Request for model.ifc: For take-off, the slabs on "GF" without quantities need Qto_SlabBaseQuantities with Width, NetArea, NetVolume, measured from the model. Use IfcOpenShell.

First a look at what the model holds.

```python
import ifcopenshell
import ifcopenshell.util.element
import ifcopenshell.util.unit

model = ifcopenshell.open("model.ifc")
print(model.schema)
for unit_type in ("LENGTHUNIT", "AREAUNIT", "VOLUMEUNIT"):
    print(unit_type, ifcopenshell.util.unit.calculate_unit_scale(model, unit_type))
storey = next(s for s in model.by_type("IfcBuildingStorey") if s.Name == "GF")
slabs = [e for e in ifcopenshell.util.element.get_decomposition(storey) if e.is_a("IfcSlab")]
for e in sorted(slabs, key=lambda e: e.id()):
    print(e.id(), e.is_a(), e.Name, list(ifcopenshell.util.element.get_psets(e, qtos_only=True)), sep=" | ")
```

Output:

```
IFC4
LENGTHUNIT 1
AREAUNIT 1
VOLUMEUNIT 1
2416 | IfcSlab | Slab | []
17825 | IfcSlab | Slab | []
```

```python
import ifcopenshell
import ifcopenshell.api.pset
import ifcopenshell.geom
import ifcopenshell.util.element
import ifcopenshell.util.shape
import ifcopenshell.util.unit

model = ifcopenshell.open("model.ifc")
unit_scale = ifcopenshell.util.unit.calculate_unit_scale(model)
area_scale = ifcopenshell.util.unit.calculate_unit_scale(model, "AREAUNIT")
volume_scale = ifcopenshell.util.unit.calculate_unit_scale(model, "VOLUMEUNIT")
settings = ifcopenshell.geom.settings()

storey = next(s for s in model.by_type("IfcBuildingStorey") if s.Name == "GF")
slabs = [e for e in ifcopenshell.util.element.get_decomposition(storey) if e.is_a("IfcSlab")]

for e in sorted(slabs, key=lambda e: e.id()):
    if ifcopenshell.util.element.get_psets(e, qtos_only=True, should_inherit=False):
        continue
    # Geometry comes back in metres, in the element's own axes.
    shape = ifcopenshell.geom.create_shape(settings, e)
    values = {
        "Width": ifcopenshell.util.shape.get_z(shape.geometry) / unit_scale,
        "NetArea": ifcopenshell.util.shape.get_footprint_area(shape.geometry) / area_scale,
        "NetVolume": ifcopenshell.util.shape.get_volume(shape.geometry) / volume_scale,
    }
    qto = ifcopenshell.api.pset.add_qto(model, product=e, name="Qto_SlabBaseQuantities")
    ifcopenshell.api.pset.edit_qto(model, qto=qto, properties=values)
    print(e.id(), {k: round(v, 3) for k, v in values.items()})

model.write("model_edited.ifc")
```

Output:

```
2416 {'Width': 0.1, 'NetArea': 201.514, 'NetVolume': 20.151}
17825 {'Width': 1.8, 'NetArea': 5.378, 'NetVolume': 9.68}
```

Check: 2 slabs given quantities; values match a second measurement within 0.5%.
